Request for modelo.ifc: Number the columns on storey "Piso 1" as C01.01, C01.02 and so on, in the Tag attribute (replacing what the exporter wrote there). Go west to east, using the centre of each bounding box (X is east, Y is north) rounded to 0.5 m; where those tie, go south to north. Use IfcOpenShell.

First a look at what the model holds.

```python
import ifcopenshell
import ifcopenshell.util.element
import ifcopenshell.util.placement

model = ifcopenshell.open("modelo.ifc")
print(model.schema)
storey = next(s for s in model.by_type("IfcBuildingStorey") if s.Name == "Piso 1")
columns = [e for e in ifcopenshell.util.element.get_decomposition(storey) if e.is_a("IfcColumn")]
for e in sorted(columns, key=lambda e: e.id()):
    origin = ifcopenshell.util.placement.get_local_placement(e.ObjectPlacement)[:3, 3]
    print(e.id(), e.Tag, e.Name, origin.round(2) + 0.0, sep=" | ")
```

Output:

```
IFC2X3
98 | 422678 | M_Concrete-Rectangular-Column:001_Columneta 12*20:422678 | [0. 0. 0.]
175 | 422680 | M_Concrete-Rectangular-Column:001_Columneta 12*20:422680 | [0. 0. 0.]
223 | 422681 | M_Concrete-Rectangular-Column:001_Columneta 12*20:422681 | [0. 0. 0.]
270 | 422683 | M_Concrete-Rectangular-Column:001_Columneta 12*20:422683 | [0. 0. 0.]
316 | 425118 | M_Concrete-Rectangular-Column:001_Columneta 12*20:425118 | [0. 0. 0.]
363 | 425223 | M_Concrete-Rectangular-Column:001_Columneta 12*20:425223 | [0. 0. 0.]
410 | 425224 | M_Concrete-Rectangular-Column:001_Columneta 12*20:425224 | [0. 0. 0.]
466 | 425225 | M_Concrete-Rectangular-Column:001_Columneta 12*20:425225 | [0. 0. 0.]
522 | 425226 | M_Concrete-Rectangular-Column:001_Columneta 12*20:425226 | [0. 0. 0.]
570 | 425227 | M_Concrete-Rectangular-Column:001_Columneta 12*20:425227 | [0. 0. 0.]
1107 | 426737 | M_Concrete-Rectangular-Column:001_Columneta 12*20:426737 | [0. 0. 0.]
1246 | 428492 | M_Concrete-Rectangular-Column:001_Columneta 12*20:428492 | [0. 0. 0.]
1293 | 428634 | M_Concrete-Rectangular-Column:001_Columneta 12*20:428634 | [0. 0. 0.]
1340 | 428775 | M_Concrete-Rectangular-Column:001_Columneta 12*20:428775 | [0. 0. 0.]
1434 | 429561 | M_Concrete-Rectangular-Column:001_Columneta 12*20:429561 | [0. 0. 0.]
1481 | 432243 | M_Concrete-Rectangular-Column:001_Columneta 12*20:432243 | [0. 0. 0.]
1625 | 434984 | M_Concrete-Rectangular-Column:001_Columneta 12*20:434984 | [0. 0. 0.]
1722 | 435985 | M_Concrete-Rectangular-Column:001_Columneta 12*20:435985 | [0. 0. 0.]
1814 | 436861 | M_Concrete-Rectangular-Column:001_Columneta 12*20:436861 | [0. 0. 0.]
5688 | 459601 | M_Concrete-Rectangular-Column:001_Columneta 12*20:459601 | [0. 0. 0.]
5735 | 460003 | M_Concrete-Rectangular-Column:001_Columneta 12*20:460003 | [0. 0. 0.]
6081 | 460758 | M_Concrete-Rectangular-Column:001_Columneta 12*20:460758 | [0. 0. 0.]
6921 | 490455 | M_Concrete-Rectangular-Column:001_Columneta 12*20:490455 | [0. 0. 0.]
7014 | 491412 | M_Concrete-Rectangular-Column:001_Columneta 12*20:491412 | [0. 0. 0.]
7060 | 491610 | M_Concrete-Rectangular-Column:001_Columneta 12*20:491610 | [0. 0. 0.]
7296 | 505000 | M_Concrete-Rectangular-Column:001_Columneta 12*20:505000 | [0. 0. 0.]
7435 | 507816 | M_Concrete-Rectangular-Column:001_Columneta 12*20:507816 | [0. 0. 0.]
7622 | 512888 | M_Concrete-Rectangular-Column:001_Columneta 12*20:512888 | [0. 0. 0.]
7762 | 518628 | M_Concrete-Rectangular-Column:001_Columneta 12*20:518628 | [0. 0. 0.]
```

```python
import ifcopenshell
import ifcopenshell.geom
import ifcopenshell.util.element
import ifcopenshell.util.shape

model = ifcopenshell.open("modelo.ifc")
settings = ifcopenshell.geom.settings()
settings.set("use-world-coords", True)


def centre(element):
    shape = ifcopenshell.geom.create_shape(settings, element)
    return ifcopenshell.util.shape.get_bbox_centroid(shape.geometry)


storey = next(s for s in model.by_type("IfcBuildingStorey") if s.Name == "Piso 1")
columns = [e for e in ifcopenshell.util.element.get_decomposition(storey) if e.is_a("IfcColumn")]

# Insertion points can sit at a corner or the storey origin, so sort by the geometry (in metres).
centres = {e: centre(e) for e in columns}
columns.sort(key=lambda e: (round(centres[e][0] / 0.5), centres[e][1]))

for i, e in enumerate(columns, start=1):
    number = f"C01.{i:02d}"
    e.Tag = number
    print(e.id(), number)

model.write("modelo_updated.ifc")
```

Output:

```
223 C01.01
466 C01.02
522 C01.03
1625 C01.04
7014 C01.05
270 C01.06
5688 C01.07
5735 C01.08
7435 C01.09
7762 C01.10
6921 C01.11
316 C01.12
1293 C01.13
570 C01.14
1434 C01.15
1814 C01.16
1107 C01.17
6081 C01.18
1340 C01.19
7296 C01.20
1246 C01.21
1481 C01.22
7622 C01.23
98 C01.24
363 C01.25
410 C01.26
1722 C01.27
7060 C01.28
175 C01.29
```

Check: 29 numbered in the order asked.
